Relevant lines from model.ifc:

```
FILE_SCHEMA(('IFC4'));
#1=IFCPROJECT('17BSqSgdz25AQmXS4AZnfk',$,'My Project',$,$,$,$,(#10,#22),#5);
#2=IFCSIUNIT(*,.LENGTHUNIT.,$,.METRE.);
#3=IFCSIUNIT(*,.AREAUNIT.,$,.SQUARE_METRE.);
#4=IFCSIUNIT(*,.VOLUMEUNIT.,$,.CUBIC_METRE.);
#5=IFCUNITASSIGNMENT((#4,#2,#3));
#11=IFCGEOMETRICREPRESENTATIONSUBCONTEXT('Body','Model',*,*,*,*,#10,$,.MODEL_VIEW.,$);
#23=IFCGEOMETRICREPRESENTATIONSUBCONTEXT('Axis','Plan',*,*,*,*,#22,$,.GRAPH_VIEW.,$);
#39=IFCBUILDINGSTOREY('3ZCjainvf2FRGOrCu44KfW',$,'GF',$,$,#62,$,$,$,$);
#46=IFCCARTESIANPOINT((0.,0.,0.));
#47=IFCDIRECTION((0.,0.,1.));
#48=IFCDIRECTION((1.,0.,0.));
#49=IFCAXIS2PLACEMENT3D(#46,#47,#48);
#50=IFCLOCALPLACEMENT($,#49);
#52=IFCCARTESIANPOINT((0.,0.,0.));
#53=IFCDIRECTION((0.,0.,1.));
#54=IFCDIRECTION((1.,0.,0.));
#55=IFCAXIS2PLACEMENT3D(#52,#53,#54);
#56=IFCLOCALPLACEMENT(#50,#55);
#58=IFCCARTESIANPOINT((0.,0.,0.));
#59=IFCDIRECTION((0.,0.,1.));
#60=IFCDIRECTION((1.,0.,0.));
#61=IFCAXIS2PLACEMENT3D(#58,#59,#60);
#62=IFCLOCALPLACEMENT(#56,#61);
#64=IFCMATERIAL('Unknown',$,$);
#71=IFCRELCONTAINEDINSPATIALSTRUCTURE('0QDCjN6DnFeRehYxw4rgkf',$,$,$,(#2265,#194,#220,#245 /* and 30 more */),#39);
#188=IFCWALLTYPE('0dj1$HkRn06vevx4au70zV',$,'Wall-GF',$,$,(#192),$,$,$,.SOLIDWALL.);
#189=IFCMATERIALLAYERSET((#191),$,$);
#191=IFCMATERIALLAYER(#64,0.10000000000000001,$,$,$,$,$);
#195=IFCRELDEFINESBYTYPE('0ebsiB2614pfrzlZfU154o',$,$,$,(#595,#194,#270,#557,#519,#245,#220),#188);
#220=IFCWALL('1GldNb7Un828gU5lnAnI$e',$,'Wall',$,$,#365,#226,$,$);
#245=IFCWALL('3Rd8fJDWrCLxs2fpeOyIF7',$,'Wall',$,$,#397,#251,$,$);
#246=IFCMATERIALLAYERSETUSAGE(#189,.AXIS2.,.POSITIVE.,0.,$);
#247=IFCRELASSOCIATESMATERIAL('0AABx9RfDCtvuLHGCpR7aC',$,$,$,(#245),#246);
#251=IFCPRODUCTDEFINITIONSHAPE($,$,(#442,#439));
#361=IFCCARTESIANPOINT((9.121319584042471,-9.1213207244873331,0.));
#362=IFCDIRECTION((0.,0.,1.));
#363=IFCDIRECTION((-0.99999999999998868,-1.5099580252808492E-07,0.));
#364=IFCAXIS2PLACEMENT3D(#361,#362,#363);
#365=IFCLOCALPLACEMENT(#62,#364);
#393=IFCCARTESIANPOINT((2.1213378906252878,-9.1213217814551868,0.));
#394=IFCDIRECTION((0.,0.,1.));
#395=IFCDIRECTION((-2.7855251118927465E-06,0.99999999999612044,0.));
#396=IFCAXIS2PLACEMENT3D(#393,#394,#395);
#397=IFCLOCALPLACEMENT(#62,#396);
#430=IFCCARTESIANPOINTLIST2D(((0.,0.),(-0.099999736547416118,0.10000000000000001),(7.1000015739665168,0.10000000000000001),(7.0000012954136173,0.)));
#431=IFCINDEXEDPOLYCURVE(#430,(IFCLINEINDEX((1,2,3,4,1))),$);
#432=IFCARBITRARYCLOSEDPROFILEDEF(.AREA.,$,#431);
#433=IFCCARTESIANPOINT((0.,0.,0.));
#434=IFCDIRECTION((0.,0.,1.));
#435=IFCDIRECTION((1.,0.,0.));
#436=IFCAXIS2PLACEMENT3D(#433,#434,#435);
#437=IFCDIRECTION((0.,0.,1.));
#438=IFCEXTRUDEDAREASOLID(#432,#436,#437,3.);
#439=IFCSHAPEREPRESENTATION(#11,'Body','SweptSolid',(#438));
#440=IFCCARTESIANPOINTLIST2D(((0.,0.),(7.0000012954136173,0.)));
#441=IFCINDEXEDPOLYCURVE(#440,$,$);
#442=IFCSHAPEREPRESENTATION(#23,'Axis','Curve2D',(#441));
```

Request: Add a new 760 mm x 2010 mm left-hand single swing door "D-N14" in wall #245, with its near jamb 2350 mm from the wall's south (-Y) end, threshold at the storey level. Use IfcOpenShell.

```python
import numpy as np
import ifcopenshell
import ifcopenshell.api.feature
import ifcopenshell.api.geometry
import ifcopenshell.api.root
import ifcopenshell.api.spatial
import ifcopenshell.geom
import ifcopenshell.util.element
import ifcopenshell.util.placement
import ifcopenshell.util.representation
import ifcopenshell.util.shape
import ifcopenshell.util.unit

model = ifcopenshell.open("model.ifc")
unit_scale = ifcopenshell.util.unit.calculate_unit_scale(model)
settings = ifcopenshell.geom.settings()


def volume(element):
    """Net volume in cubic metres, openings subtracted."""
    shape = ifcopenshell.geom.create_shape(settings, element)
    return ifcopenshell.util.shape.get_volume(shape.geometry)


wall = model.by_guid("3Rd8fJDWrCLxs2fpeOyIF7")
storey = ifcopenshell.util.element.get_container(wall, ifc_class="IfcBuildingStorey")
context = ifcopenshell.util.representation.get_context(model, "Model", "Body", "MODEL_VIEW")
before = volume(wall)

width, height, from_end, sill = 0.76, 2.01, 2.35, 0.0  # metres

# The wall runs along its own X axis, and the end named is its -X end.
wall_shape = ifcopenshell.geom.create_shape(settings, wall)
x, y, z = ifcopenshell.util.shape.get_vertices(wall_shape.geometry).T
start = x.min() + from_end
face, thickness = float(y.min()), float(y.max() - y.min())
wall_matrix = ifcopenshell.util.placement.get_local_placement(wall.ObjectPlacement)
level = ifcopenshell.util.placement.get_local_placement(storey.ObjectPlacement)[2, 3]


def in_wall(x, y):
    """Placement at x, y metres in the wall's axes, at sill height."""
    matrix = wall_matrix.copy()
    matrix[:, 3] = wall_matrix @ np.array([x / unit_scale, y / unit_scale, 0.0, 1.0])
    matrix[2, 3] = level + sill / unit_scale
    return matrix


# Opening: a box that overshoots both wall faces by 50 mm.
opening = ifcopenshell.api.root.create_entity(model, ifc_class="IfcOpeningElement", predefined_type="OPENING")
box = ifcopenshell.api.geometry.add_wall_representation(
    model, context=context, length=width, height=height, thickness=thickness + 0.1
)
ifcopenshell.api.geometry.assign_representation(model, product=opening, representation=box)
ifcopenshell.api.geometry.edit_object_placement(model, product=opening, matrix=in_wall(start, face - 0.05), is_si=False)
ifcopenshell.api.feature.add_feature(model, feature=opening, element=wall)

door = ifcopenshell.api.root.create_entity(model, ifc_class="IfcDoor", name="D-N14", predefined_type="DOOR")
door.OverallWidth, door.OverallHeight = width / unit_scale, height / unit_scale
door.OperationType = "SINGLE_SWING_LEFT"
body = ifcopenshell.api.geometry.add_door_representation(
    model,
    context=context,
    overall_width=door.OverallWidth,
    overall_height=door.OverallHeight,
    operation_type="SINGLE_SWING_LEFT",
    lining_properties={"LiningDepth": thickness / unit_scale, "ThresholdDepth": thickness / unit_scale},
)
ifcopenshell.api.geometry.assign_representation(model, product=door, representation=body)
ifcopenshell.api.spatial.assign_container(model, products=[door], relating_structure=storey)
ifcopenshell.api.feature.add_filling(model, opening=opening, element=door)

# The lining spans the wall, so the door starts at the wall face.
ifcopenshell.api.geometry.edit_object_placement(model, product=door, matrix=in_wall(start, face), is_si=False)

after = volume(wall)

print(f"wall volume {before:.3f} -> {after:.3f} m3")

model.write("model_edited.ifc")
```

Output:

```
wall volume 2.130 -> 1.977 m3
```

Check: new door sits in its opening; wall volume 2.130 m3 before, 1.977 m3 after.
